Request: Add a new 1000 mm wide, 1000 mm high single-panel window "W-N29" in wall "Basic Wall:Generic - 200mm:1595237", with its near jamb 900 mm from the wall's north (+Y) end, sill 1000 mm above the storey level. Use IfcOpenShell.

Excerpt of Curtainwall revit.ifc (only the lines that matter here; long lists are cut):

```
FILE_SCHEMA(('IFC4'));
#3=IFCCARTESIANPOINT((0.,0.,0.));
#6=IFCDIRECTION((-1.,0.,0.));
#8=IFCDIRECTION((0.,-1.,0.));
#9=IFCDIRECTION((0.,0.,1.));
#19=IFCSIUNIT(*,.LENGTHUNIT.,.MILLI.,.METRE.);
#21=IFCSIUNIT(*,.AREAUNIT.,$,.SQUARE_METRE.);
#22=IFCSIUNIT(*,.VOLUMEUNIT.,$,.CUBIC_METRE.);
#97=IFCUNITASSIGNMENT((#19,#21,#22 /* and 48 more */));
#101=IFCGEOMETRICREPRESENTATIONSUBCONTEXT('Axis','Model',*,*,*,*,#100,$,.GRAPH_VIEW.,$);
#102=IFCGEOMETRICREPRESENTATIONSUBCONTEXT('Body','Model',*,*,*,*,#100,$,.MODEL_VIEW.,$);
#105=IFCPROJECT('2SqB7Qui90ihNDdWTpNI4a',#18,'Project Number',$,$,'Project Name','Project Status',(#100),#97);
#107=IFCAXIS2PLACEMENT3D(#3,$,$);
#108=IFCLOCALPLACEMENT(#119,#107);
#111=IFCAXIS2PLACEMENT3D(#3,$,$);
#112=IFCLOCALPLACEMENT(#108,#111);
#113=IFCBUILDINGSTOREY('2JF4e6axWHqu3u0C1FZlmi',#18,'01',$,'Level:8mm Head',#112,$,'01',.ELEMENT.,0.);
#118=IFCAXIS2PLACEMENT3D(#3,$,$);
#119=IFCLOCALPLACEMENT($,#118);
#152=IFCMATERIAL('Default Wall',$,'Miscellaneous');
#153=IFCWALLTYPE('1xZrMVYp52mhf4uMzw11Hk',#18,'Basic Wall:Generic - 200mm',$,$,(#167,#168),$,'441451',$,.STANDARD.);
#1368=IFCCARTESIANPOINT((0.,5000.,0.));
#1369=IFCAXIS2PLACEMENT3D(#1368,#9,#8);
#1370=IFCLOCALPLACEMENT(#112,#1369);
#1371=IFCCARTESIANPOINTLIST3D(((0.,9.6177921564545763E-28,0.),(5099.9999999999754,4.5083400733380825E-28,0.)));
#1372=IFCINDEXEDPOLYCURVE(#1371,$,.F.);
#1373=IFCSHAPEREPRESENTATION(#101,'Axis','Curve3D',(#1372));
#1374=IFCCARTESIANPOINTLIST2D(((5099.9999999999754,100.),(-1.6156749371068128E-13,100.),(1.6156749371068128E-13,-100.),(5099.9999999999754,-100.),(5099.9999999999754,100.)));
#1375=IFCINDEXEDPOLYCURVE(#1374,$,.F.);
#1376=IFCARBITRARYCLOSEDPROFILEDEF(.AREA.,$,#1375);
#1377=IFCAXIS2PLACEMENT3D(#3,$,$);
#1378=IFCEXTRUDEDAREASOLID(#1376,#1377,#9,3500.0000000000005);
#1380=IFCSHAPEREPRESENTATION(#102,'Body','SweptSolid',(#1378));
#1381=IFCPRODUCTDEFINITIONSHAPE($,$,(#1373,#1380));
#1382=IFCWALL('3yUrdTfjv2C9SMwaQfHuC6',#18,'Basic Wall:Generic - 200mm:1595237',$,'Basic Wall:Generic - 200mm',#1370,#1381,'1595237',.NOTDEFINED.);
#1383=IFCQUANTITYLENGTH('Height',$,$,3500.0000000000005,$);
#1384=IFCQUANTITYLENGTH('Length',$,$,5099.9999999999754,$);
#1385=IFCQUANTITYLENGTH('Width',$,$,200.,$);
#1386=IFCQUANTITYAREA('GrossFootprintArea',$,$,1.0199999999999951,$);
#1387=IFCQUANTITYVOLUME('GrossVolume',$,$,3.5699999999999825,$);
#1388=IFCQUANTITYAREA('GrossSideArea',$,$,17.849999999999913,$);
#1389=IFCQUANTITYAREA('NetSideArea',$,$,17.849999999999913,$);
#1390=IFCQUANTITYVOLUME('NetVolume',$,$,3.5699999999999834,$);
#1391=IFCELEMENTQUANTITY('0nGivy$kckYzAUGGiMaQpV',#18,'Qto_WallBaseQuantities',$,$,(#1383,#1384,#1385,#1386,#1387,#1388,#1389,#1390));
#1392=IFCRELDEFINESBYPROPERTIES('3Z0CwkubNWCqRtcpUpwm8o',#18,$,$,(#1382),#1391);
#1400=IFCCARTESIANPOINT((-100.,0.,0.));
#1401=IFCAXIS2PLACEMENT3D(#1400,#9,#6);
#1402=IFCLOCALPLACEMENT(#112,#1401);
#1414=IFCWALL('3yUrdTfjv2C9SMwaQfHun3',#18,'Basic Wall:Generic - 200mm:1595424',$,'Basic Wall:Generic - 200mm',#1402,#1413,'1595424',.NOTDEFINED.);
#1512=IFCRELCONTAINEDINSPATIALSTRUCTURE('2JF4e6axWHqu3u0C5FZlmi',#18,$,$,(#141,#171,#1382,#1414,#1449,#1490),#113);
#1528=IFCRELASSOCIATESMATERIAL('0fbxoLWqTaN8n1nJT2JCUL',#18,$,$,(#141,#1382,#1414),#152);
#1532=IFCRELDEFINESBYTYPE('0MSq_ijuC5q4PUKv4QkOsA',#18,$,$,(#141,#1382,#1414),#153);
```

```python
import numpy as np
import ifcopenshell
import ifcopenshell.api.feature
import ifcopenshell.api.geometry
import ifcopenshell.api.pset
import ifcopenshell.api.root
import ifcopenshell.api.spatial
import ifcopenshell.geom
import ifcopenshell.util.element
import ifcopenshell.util.placement
import ifcopenshell.util.representation
import ifcopenshell.util.shape
import ifcopenshell.util.unit

model = ifcopenshell.open("Curtainwall revit.ifc")
unit_scale = ifcopenshell.util.unit.calculate_unit_scale(model)
area_scale = ifcopenshell.util.unit.calculate_unit_scale(model, "AREAUNIT")
volume_scale = ifcopenshell.util.unit.calculate_unit_scale(model, "VOLUMEUNIT")
settings = ifcopenshell.geom.settings()


def volume(element):
    """Net volume in cubic metres, openings subtracted."""
    shape = ifcopenshell.geom.create_shape(settings, element)
    return ifcopenshell.util.shape.get_volume(shape.geometry)


wall = model.by_guid("3yUrdTfjv2C9SMwaQfHuC6")
storey = ifcopenshell.util.element.get_container(wall, ifc_class="IfcBuildingStorey")
context = ifcopenshell.util.representation.get_context(model, "Model", "Body", "MODEL_VIEW")
before = volume(wall)

width, height, from_end, sill = 1, 1, 0.9, 1  # metres

# The wall runs along its own X axis, and the end named is its -X end.
wall_shape = ifcopenshell.geom.create_shape(settings, wall)
x, y, z = ifcopenshell.util.shape.get_vertices(wall_shape.geometry).T
start = x.min() + from_end
face, thickness = float(y.min()), float(y.max() - y.min())
wall_matrix = ifcopenshell.util.placement.get_local_placement(wall.ObjectPlacement)
level = ifcopenshell.util.placement.get_local_placement(storey.ObjectPlacement)[2, 3]


def in_wall(x, y):
    """Placement at x, y metres in the wall's axes, at sill height."""
    matrix = wall_matrix.copy()
    matrix[:, 3] = wall_matrix @ np.array([x / unit_scale, y / unit_scale, 0.0, 1.0])
    matrix[2, 3] = level + sill / unit_scale
    return matrix


# Opening: a box that overshoots both wall faces by 50 mm.
opening = ifcopenshell.api.root.create_entity(model, ifc_class="IfcOpeningElement", predefined_type="OPENING")
box = ifcopenshell.api.geometry.add_wall_representation(
    model, context=context, length=width, height=height, thickness=thickness + 0.1
)
ifcopenshell.api.geometry.assign_representation(model, product=opening, representation=box)
ifcopenshell.api.geometry.edit_object_placement(model, product=opening, matrix=in_wall(start, face - 0.05), is_si=False)
ifcopenshell.api.feature.add_feature(model, feature=opening, element=wall)

window = ifcopenshell.api.root.create_entity(model, ifc_class="IfcWindow", name="W-N29", predefined_type="WINDOW")
window.OverallWidth, window.OverallHeight = width / unit_scale, height / unit_scale
window.PartitioningType = "SINGLE_PANEL"
body = ifcopenshell.api.geometry.add_window_representation(
    model,
    context=context,
    overall_width=window.OverallWidth,
    overall_height=window.OverallHeight,
    partition_type="SINGLE_PANEL",
)
ifcopenshell.api.geometry.assign_representation(model, product=window, representation=body)
ifcopenshell.api.spatial.assign_container(model, products=[window], relating_structure=storey)
ifcopenshell.api.feature.add_filling(model, opening=opening, element=window)

# Centre the window in the wall's thickness.
ifcopenshell.api.geometry.edit_object_placement(model, product=window, matrix=in_wall(start, face), is_si=False)
window_shape = ifcopenshell.geom.create_shape(settings, window)
depth = ifcopenshell.util.shape.get_vertices(window_shape.geometry)[:, 1]
offset = face + thickness / 2 - (depth.min() + depth.max()) / 2
ifcopenshell.api.geometry.edit_object_placement(model, product=window, matrix=in_wall(start, offset), is_si=False)

after = volume(wall)

# Update the wall's stored quantities.
qto = model.by_id(ifcopenshell.util.element.get_pset(wall, "Qto_WallBaseQuantities", should_inherit=False)["id"])
ifcopenshell.api.pset.edit_qto(model, qto=qto, properties={
    "NetSideArea": after / thickness / area_scale,
    "NetVolume": after / volume_scale,
})

print(f"wall volume {before:.3f} -> {after:.3f} m3")

model.write("Curtainwall revit_updated.ifc")
```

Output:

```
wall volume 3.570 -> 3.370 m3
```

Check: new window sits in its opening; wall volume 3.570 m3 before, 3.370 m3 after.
